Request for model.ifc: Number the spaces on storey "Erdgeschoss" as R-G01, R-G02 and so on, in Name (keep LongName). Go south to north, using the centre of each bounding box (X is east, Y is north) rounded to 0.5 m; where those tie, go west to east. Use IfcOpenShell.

First a look at what the model holds.

```python
import ifcopenshell
import ifcopenshell.util.element
import ifcopenshell.util.placement

model = ifcopenshell.open("model.ifc")
print(model.schema)
storey = next(s for s in model.by_type("IfcBuildingStorey") if s.Name == "Erdgeschoss")
spaces = [e for e in ifcopenshell.util.element.get_decomposition(storey) if e.is_a("IfcSpace")]
for e in sorted(spaces, key=lambda e: e.id()):
    origin = ifcopenshell.util.placement.get_local_placement(e.ObjectPlacement)[:3, 3]
    print(e.id(), e.Name, e.LongName, origin.round(2) + 0.0, sep=" | ")
```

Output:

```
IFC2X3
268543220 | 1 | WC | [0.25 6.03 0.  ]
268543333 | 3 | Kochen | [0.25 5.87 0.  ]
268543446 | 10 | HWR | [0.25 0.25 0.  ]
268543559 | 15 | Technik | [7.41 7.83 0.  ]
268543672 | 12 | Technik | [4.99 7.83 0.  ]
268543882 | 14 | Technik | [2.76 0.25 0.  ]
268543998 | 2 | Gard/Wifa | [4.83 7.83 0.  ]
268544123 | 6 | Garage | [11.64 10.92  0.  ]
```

```python
import ifcopenshell
import ifcopenshell.geom
import ifcopenshell.util.element
import ifcopenshell.util.shape

model = ifcopenshell.open("model.ifc")
settings = ifcopenshell.geom.settings()
settings.set("use-world-coords", True)


def centre(element):
    shape = ifcopenshell.geom.create_shape(settings, element)
    return ifcopenshell.util.shape.get_bbox_centroid(shape.geometry)


storey = next(s for s in model.by_type("IfcBuildingStorey") if s.Name == "Erdgeschoss")
spaces = [e for e in ifcopenshell.util.element.get_decomposition(storey) if e.is_a("IfcSpace")]

# Insertion points can sit at a corner or the storey origin, so sort by the geometry (in metres).
centres = {e: centre(e) for e in spaces}
spaces.sort(key=lambda e: (round(centres[e][1] / 0.5), centres[e][0]))

for i, e in enumerate(spaces, start=1):
    number = f"R-G{i:02d}"
    e.Name = number
    print(e.id(), number)

model.write("model_v2.ifc")
```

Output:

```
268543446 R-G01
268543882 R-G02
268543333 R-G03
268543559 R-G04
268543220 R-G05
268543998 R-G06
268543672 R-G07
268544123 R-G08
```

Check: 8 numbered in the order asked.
